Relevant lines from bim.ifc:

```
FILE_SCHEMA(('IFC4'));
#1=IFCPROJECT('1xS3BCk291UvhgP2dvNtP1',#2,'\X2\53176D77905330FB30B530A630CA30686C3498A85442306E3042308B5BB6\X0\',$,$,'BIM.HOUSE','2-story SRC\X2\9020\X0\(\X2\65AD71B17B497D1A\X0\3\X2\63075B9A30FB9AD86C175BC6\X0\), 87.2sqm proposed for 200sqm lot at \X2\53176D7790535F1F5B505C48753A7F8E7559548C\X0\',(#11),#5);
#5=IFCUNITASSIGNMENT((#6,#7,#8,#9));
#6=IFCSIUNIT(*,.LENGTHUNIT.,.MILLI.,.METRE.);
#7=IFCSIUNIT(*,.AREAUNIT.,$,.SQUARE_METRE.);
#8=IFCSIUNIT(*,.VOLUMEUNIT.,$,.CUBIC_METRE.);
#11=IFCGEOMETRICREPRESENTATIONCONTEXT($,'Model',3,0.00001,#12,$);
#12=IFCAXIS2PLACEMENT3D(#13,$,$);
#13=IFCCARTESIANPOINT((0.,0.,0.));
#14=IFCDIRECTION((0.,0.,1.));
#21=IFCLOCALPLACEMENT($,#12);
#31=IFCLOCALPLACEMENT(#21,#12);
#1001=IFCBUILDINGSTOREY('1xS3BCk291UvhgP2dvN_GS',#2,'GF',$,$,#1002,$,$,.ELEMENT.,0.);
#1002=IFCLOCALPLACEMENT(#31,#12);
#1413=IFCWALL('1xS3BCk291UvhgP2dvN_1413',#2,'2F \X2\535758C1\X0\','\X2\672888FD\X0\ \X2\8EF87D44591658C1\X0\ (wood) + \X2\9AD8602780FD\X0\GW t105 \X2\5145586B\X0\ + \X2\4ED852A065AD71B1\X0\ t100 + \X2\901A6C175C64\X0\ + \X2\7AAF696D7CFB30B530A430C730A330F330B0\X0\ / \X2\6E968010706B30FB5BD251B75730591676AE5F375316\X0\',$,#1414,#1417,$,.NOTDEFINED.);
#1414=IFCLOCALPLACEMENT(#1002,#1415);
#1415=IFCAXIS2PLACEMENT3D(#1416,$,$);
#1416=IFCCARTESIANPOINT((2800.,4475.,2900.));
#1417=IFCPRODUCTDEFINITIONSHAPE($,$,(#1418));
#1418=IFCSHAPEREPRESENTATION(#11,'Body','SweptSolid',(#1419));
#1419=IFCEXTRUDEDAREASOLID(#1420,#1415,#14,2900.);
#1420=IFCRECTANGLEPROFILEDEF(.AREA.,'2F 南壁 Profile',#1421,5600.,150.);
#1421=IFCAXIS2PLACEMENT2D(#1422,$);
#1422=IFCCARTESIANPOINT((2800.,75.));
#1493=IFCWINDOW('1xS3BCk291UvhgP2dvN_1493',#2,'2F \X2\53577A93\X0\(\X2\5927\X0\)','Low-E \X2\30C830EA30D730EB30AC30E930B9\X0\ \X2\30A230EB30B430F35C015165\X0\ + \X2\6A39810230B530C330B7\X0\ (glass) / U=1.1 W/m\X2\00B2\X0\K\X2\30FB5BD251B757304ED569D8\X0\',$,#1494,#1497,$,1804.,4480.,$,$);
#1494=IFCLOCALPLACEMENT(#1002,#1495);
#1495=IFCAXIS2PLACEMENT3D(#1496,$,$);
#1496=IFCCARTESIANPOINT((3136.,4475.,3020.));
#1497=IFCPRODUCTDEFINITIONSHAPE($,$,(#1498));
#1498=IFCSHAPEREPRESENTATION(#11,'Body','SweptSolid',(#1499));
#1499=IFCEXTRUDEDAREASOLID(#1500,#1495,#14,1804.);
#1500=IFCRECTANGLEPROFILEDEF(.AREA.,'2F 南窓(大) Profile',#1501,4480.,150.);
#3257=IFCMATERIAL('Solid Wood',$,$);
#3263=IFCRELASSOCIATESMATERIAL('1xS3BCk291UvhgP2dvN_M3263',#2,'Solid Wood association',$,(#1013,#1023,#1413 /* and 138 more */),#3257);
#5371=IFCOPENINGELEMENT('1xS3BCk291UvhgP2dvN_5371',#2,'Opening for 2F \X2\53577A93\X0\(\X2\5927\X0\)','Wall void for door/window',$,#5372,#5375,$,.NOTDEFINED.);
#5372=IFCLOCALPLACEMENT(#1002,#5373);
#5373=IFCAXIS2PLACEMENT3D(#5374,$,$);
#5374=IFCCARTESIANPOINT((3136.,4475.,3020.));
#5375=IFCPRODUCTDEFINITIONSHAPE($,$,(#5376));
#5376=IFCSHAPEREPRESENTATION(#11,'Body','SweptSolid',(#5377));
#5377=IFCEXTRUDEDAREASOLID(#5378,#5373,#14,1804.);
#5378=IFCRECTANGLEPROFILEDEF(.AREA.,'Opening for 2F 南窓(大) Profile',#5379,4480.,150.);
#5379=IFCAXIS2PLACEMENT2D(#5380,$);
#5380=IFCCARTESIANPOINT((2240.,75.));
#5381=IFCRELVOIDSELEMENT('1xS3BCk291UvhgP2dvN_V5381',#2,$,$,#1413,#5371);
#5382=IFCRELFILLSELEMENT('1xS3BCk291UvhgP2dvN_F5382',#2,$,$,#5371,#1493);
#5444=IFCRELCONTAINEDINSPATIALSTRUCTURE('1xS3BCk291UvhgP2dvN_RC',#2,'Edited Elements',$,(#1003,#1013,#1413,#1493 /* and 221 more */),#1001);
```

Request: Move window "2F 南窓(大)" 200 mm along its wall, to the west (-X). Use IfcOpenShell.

```python
import ifcopenshell
import ifcopenshell.api.geometry
import ifcopenshell.util.placement

model = ifcopenshell.open("bim.ifc")

window = model.by_guid("1xS3BCk291UvhgP2dvN_1493")
opening = window.FillsVoids[0].RelatingOpeningElement
wall = opening.VoidsElements[0].RelatingBuildingElement

wall_matrix = ifcopenshell.util.placement.get_local_placement(wall.ObjectPlacement)
shift = wall_matrix[:3, 0] * -200.0
before = ifcopenshell.util.placement.get_local_placement(window.ObjectPlacement)[:3, 3].copy()

# The window is not placed relative to its opening, so move both.
for product in (opening, window):
    matrix = ifcopenshell.util.placement.get_local_placement(product.ObjectPlacement)
    matrix[:3, 3] += shift
    ifcopenshell.api.geometry.edit_object_placement(model, product=product, matrix=matrix, is_si=False)

after = ifcopenshell.util.placement.get_local_placement(window.ObjectPlacement)[:3, 3]
print("window moved by", (after - before).round(3) + 0.0)

model.write("bim_updated.ifc")
```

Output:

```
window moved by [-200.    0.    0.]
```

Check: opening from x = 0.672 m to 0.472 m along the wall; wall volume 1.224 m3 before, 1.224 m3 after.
